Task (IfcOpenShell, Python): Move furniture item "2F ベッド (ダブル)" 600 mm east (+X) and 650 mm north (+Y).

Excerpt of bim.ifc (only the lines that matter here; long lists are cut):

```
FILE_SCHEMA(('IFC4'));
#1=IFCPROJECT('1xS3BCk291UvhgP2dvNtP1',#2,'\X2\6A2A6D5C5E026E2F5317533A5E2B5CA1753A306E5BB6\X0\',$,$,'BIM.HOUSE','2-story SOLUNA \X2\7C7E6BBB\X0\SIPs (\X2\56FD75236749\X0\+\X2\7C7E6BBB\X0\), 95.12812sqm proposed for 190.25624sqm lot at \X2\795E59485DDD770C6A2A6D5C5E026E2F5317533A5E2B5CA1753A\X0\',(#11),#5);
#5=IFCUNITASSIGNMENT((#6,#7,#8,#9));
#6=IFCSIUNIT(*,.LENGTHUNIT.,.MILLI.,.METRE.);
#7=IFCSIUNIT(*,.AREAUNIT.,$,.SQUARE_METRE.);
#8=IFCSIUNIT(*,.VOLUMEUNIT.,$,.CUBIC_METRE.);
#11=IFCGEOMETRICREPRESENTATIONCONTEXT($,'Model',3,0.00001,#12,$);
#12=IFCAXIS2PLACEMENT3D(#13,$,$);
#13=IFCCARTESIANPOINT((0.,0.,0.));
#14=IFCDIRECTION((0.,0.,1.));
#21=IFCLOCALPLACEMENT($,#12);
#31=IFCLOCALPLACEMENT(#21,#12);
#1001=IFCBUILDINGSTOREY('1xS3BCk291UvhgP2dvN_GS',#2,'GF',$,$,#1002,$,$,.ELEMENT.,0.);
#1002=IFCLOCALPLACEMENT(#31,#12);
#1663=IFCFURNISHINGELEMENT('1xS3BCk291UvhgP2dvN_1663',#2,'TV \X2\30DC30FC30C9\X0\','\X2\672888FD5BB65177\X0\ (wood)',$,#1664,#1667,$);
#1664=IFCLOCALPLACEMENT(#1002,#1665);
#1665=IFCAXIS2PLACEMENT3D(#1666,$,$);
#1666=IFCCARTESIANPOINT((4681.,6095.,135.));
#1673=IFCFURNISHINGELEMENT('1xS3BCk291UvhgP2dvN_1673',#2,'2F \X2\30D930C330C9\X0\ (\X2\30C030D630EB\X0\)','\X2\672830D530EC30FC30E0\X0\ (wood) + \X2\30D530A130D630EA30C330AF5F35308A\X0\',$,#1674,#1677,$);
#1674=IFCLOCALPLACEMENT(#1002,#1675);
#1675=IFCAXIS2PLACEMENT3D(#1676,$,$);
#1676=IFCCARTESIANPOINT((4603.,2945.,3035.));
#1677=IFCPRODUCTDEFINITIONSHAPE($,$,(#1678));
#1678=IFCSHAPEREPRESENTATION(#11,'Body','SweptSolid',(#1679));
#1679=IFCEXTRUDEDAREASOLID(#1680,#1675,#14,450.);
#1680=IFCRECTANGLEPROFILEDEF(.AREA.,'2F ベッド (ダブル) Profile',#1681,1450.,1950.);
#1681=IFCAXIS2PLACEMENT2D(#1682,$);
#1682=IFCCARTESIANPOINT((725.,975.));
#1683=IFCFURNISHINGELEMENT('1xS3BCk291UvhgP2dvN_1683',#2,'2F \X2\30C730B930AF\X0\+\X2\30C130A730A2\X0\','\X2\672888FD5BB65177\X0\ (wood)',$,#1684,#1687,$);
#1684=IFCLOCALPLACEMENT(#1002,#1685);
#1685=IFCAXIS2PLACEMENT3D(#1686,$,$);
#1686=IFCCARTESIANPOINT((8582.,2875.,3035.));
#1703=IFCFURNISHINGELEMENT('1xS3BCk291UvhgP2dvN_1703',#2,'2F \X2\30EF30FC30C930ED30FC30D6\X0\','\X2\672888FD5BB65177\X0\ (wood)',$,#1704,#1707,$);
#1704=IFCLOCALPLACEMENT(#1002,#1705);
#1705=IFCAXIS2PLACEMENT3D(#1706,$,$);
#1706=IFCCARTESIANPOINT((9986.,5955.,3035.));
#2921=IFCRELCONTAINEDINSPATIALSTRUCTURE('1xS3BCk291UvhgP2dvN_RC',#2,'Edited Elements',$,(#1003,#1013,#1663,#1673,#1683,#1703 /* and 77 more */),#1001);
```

```python
import ifcopenshell
import ifcopenshell.api.geometry
import ifcopenshell.util.placement

model = ifcopenshell.open("bim.ifc")

item = model.by_guid("1xS3BCk291UvhgP2dvN_1673")
matrix = ifcopenshell.util.placement.get_local_placement(item.ObjectPlacement)
matrix[0, 3] += 600.0
matrix[1, 3] += 650.0
ifcopenshell.api.geometry.edit_object_placement(model, product=item, matrix=matrix, is_si=False)

print(ifcopenshell.util.placement.get_local_placement(item.ObjectPlacement).round(3) + 0.0)

model.write("bim_edited.ifc")
```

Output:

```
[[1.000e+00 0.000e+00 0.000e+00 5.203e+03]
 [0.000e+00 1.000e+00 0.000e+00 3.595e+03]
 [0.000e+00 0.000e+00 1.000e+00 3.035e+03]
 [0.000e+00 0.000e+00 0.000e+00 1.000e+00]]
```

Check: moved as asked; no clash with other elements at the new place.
